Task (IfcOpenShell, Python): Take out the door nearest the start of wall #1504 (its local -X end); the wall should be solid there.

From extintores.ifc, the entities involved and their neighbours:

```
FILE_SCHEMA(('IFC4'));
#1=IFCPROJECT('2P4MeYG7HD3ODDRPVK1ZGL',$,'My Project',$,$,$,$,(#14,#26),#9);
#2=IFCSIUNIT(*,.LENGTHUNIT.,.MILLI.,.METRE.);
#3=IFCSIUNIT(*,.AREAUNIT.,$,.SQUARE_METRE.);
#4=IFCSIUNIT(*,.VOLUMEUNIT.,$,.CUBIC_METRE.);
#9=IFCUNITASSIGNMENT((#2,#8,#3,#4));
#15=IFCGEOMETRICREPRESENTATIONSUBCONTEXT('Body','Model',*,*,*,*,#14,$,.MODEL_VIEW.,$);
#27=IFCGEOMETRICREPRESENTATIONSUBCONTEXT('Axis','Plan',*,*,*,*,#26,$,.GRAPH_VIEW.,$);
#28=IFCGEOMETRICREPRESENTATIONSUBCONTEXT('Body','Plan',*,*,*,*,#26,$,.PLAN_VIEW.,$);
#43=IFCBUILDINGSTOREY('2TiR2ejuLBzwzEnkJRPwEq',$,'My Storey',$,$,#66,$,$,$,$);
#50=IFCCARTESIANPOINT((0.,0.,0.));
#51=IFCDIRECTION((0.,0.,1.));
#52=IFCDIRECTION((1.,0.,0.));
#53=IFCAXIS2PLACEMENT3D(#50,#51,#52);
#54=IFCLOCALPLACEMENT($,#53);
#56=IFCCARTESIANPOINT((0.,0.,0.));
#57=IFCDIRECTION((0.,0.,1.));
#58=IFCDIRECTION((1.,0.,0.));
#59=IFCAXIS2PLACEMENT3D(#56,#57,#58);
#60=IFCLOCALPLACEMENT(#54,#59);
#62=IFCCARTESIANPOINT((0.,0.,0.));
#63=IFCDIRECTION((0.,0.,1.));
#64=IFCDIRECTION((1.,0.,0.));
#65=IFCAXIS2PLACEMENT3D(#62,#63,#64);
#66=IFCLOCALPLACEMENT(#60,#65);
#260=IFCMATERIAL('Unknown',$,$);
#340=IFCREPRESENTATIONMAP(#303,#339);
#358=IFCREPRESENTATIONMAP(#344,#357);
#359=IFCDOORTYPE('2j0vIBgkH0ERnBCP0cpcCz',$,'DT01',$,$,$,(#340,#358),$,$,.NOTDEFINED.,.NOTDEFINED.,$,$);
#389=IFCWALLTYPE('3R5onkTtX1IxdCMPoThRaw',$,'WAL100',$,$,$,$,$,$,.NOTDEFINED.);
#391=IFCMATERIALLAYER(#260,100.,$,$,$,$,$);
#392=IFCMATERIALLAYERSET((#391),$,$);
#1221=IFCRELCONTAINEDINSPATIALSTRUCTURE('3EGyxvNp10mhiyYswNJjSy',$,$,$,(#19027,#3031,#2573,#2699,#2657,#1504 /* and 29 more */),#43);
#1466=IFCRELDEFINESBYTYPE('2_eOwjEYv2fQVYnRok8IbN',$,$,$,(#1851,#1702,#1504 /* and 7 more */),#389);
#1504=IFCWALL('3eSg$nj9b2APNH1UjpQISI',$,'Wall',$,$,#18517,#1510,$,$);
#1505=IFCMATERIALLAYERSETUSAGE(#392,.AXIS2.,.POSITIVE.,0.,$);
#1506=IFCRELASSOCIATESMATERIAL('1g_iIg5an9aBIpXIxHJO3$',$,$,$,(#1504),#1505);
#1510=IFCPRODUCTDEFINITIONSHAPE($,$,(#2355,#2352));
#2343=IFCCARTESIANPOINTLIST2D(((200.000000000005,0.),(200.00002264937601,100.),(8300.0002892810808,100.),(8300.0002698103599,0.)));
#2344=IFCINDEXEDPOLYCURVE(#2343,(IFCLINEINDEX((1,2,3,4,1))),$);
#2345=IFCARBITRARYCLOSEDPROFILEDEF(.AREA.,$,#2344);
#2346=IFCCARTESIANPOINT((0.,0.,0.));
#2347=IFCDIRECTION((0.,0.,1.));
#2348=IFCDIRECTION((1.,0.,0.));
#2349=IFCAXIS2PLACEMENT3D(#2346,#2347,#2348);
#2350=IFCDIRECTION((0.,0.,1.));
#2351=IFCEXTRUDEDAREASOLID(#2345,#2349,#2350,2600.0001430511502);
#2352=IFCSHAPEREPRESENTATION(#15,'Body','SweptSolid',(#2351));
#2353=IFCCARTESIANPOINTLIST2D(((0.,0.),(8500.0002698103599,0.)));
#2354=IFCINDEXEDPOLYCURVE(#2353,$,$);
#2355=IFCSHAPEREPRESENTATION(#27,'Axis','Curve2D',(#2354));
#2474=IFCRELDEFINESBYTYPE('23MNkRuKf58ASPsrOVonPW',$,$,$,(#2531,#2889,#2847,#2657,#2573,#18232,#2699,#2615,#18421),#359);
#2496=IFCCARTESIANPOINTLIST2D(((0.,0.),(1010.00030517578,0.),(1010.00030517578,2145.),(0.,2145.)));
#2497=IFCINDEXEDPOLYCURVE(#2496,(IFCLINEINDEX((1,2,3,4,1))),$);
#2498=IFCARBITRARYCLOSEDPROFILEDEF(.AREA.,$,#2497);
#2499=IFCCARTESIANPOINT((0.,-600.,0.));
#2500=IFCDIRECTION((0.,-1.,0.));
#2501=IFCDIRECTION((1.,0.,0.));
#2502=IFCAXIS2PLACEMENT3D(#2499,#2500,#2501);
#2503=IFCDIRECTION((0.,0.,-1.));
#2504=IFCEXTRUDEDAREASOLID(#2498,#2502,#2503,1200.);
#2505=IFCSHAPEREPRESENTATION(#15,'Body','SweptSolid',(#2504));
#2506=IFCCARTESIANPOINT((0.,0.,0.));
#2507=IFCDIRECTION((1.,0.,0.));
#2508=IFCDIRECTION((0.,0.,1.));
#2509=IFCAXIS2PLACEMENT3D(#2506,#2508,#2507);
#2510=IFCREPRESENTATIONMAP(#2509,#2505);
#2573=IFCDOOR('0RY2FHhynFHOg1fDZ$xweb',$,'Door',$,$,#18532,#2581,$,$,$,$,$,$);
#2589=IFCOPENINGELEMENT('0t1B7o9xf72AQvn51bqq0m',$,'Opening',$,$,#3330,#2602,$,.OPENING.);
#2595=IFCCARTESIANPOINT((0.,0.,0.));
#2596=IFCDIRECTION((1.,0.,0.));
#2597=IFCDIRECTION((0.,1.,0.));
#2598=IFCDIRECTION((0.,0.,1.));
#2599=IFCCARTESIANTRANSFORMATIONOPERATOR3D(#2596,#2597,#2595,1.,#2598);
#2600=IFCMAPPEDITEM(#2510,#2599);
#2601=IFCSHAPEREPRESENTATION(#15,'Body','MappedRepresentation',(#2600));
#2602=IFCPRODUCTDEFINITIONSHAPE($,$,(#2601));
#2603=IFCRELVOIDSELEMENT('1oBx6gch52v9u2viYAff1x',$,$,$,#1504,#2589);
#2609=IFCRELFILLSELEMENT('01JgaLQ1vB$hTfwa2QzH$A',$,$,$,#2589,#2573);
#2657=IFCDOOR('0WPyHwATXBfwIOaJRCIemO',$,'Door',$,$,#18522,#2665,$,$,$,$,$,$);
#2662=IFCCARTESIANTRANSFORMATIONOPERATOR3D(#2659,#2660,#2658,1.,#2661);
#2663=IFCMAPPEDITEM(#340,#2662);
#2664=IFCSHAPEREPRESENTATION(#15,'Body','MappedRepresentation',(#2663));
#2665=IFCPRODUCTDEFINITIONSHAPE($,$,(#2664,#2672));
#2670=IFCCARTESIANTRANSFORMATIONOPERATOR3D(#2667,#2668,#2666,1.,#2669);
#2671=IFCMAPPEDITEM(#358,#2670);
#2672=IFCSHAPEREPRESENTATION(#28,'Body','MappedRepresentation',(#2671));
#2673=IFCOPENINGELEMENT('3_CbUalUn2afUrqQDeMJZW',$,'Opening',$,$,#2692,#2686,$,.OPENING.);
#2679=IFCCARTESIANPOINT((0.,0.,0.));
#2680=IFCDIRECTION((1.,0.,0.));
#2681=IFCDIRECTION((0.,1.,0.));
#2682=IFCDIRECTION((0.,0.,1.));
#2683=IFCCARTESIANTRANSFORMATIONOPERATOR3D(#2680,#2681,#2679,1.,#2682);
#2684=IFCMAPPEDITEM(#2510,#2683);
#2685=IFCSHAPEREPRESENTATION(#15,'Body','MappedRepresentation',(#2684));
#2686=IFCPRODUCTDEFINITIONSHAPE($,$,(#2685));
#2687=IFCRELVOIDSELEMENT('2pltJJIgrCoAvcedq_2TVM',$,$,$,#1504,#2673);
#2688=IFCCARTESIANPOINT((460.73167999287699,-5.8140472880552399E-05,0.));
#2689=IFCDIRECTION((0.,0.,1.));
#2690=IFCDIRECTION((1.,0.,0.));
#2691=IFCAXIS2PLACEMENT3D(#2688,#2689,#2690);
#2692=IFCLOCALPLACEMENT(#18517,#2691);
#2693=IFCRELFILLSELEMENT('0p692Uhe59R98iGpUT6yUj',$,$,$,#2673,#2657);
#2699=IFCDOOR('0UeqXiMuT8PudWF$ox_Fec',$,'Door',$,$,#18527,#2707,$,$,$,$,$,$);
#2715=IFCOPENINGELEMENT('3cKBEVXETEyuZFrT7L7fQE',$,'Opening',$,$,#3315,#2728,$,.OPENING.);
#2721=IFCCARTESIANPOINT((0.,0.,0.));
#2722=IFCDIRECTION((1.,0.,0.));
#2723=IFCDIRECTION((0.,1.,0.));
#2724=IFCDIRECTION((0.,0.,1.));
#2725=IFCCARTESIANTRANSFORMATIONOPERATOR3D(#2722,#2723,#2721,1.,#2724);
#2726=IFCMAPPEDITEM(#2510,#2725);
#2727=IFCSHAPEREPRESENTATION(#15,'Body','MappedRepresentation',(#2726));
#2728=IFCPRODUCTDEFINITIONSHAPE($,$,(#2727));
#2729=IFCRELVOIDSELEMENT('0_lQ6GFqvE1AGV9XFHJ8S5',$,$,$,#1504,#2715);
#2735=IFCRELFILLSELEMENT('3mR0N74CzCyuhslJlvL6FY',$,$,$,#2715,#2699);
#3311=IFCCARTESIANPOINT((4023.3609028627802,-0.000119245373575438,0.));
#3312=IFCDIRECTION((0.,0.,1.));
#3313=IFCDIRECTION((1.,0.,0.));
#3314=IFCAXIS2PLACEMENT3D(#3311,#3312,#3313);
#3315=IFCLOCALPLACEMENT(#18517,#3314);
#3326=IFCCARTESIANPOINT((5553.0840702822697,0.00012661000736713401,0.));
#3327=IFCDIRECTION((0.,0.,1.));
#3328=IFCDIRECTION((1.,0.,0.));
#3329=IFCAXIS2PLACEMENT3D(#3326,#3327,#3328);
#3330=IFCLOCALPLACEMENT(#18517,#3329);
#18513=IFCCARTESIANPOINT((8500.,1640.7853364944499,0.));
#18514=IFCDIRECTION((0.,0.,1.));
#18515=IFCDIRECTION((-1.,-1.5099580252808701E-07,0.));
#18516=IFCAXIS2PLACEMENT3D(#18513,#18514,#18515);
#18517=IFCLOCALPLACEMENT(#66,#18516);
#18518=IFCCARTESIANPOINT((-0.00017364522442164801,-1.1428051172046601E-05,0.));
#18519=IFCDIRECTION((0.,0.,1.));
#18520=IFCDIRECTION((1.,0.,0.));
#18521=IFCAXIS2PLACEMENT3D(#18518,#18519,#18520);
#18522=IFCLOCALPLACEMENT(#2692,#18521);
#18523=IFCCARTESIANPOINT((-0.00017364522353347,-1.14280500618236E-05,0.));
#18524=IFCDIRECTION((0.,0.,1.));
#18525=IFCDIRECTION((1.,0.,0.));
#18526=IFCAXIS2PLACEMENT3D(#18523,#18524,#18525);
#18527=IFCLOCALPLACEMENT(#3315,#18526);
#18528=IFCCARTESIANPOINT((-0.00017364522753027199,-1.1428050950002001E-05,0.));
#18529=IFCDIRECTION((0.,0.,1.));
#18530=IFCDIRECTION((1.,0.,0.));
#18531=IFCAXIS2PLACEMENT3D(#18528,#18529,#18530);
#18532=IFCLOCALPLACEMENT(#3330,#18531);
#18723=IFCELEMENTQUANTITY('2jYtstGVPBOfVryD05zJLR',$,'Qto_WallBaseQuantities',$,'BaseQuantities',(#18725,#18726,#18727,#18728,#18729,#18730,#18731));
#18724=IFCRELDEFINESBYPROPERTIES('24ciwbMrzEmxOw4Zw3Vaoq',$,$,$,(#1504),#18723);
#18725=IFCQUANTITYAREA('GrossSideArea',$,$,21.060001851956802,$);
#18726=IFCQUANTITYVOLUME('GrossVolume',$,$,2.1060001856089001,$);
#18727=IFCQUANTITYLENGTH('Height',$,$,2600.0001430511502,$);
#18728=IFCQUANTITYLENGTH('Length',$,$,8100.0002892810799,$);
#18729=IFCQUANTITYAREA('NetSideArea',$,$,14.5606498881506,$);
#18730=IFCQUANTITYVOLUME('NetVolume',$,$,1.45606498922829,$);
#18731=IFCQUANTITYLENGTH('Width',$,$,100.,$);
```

```python
import ifcopenshell
import ifcopenshell.api.feature
import ifcopenshell.api.pset
import ifcopenshell.api.root
import ifcopenshell.geom
import ifcopenshell.util.element
import ifcopenshell.util.shape
import ifcopenshell.util.unit

model = ifcopenshell.open("extintores.ifc")
area_scale = ifcopenshell.util.unit.calculate_unit_scale(model, "AREAUNIT")
volume_scale = ifcopenshell.util.unit.calculate_unit_scale(model, "VOLUMEUNIT")
settings = ifcopenshell.geom.settings()


def volume(element):
    """Net volume in cubic metres, openings subtracted."""
    shape = ifcopenshell.geom.create_shape(settings, element)
    return ifcopenshell.util.shape.get_volume(shape.geometry)


door = model.by_id(2657)
opening = door.FillsVoids[0].RelatingOpeningElement
wall = opening.VoidsElements[0].RelatingBuildingElement
before = volume(wall)

ifcopenshell.api.root.remove_product(model, product=door)
ifcopenshell.api.feature.remove_feature(model, feature=opening)

after = volume(wall)
thickness = 0.1  # wall thickness in metres

# Update the wall's stored quantities.
qto = model.by_id(ifcopenshell.util.element.get_pset(wall, "Qto_WallBaseQuantities", should_inherit=False)["id"])
ifcopenshell.api.pset.edit_qto(model, qto=qto, properties={
    "NetSideArea": after / thickness / area_scale,
    "NetVolume": after / volume_scale,
})

print(f"wall volume {before:.3f} -> {after:.3f} m3")

model.write("extintores-out.ifc")
```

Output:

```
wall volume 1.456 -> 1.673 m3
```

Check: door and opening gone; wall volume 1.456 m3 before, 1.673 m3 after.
